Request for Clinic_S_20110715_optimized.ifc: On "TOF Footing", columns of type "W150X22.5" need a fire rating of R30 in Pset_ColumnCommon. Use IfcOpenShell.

First a look at what the model holds.

```python
import ifcopenshell
import ifcopenshell.util.element

model = ifcopenshell.open("Clinic_S_20110715_optimized.ifc")
print(model.schema)
storey = next(s for s in model.by_type("IfcBuildingStorey") if s.Name == "TOF Footing")
columns = [e for e in ifcopenshell.util.element.get_decomposition(storey) if e.is_a("IfcColumn")]
seen = {}
for e in columns:
    element_type = ifcopenshell.util.element.get_type(e)
    key = (element_type.Name if element_type != e and element_type else None, ifcopenshell.util.element.get_pset(e, "Pset_ColumnCommon", "FireRating"))
    seen[key] = seen.get(key, 0) + 1
for (name, value), count in sorted(seen.items(), key=str):
    print(count, "x", name, "|", value)
```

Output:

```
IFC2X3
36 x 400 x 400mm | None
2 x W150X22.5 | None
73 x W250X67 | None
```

```python
import ifcopenshell
import ifcopenshell.api.pset
import ifcopenshell.util.element

model = ifcopenshell.open("Clinic_S_20110715_optimized.ifc")

storey = next(s for s in model.by_type("IfcBuildingStorey") if s.Name == "TOF Footing")
columns = [e for e in ifcopenshell.util.element.get_decomposition(storey) if e.is_a("IfcColumn")]

count = 0
for e in columns:
    element_type = ifcopenshell.util.element.get_type(e)
    if element_type in (None, e) or element_type.Name != "W150X22.5":
        continue
    # add_pset returns the element's existing set when there is one.
    pset = ifcopenshell.api.pset.add_pset(model, product=e, name="Pset_ColumnCommon")
    ifcopenshell.api.pset.edit_pset(model, pset=pset, properties={"FireRating": "R30"})
    count += 1

print(count, "columns updated")

model.write("Clinic_S_20110715_optimized_rev.ifc")
```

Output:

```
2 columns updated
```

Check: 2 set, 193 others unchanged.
